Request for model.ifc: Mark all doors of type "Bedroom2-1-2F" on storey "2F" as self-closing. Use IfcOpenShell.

First a look at what the model holds.

```python
import ifcopenshell
import ifcopenshell.util.element

model = ifcopenshell.open("model.ifc")
print(model.schema)
storey = next(s for s in model.by_type("IfcBuildingStorey") if s.Name == "2F")
doors = [e for e in ifcopenshell.util.element.get_decomposition(storey) if e.is_a("IfcDoor")]
seen = {}
for e in doors:
    element_type = ifcopenshell.util.element.get_type(e)
    key = (element_type.Name if element_type != e and element_type else None, ifcopenshell.util.element.get_pset(e, "Pset_DoorCommon", "SelfClosing"))
    seen[key] = seen.get(key, 0) + 1
for (name, value), count in sorted(seen.items(), key=str):
    print(count, "x", name, "|", value)
```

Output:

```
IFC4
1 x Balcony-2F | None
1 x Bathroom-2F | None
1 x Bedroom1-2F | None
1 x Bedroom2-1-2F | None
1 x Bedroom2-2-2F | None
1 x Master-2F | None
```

```python
import ifcopenshell
import ifcopenshell.api.pset
import ifcopenshell.util.element

model = ifcopenshell.open("model.ifc")

storey = next(s for s in model.by_type("IfcBuildingStorey") if s.Name == "2F")
doors = [e for e in ifcopenshell.util.element.get_decomposition(storey) if e.is_a("IfcDoor")]

count = 0
for e in doors:
    element_type = ifcopenshell.util.element.get_type(e)
    if element_type in (None, e) or element_type.Name != "Bedroom2-1-2F":
        continue
    # add_pset returns the element's existing set when there is one.
    pset = ifcopenshell.api.pset.add_pset(model, product=e, name="Pset_DoorCommon")
    ifcopenshell.api.pset.edit_pset(model, pset=pset, properties={"SelfClosing": True})
    count += 1

print(count, "doors updated")

model.write("model_updated.ifc")
```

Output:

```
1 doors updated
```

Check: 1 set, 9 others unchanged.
